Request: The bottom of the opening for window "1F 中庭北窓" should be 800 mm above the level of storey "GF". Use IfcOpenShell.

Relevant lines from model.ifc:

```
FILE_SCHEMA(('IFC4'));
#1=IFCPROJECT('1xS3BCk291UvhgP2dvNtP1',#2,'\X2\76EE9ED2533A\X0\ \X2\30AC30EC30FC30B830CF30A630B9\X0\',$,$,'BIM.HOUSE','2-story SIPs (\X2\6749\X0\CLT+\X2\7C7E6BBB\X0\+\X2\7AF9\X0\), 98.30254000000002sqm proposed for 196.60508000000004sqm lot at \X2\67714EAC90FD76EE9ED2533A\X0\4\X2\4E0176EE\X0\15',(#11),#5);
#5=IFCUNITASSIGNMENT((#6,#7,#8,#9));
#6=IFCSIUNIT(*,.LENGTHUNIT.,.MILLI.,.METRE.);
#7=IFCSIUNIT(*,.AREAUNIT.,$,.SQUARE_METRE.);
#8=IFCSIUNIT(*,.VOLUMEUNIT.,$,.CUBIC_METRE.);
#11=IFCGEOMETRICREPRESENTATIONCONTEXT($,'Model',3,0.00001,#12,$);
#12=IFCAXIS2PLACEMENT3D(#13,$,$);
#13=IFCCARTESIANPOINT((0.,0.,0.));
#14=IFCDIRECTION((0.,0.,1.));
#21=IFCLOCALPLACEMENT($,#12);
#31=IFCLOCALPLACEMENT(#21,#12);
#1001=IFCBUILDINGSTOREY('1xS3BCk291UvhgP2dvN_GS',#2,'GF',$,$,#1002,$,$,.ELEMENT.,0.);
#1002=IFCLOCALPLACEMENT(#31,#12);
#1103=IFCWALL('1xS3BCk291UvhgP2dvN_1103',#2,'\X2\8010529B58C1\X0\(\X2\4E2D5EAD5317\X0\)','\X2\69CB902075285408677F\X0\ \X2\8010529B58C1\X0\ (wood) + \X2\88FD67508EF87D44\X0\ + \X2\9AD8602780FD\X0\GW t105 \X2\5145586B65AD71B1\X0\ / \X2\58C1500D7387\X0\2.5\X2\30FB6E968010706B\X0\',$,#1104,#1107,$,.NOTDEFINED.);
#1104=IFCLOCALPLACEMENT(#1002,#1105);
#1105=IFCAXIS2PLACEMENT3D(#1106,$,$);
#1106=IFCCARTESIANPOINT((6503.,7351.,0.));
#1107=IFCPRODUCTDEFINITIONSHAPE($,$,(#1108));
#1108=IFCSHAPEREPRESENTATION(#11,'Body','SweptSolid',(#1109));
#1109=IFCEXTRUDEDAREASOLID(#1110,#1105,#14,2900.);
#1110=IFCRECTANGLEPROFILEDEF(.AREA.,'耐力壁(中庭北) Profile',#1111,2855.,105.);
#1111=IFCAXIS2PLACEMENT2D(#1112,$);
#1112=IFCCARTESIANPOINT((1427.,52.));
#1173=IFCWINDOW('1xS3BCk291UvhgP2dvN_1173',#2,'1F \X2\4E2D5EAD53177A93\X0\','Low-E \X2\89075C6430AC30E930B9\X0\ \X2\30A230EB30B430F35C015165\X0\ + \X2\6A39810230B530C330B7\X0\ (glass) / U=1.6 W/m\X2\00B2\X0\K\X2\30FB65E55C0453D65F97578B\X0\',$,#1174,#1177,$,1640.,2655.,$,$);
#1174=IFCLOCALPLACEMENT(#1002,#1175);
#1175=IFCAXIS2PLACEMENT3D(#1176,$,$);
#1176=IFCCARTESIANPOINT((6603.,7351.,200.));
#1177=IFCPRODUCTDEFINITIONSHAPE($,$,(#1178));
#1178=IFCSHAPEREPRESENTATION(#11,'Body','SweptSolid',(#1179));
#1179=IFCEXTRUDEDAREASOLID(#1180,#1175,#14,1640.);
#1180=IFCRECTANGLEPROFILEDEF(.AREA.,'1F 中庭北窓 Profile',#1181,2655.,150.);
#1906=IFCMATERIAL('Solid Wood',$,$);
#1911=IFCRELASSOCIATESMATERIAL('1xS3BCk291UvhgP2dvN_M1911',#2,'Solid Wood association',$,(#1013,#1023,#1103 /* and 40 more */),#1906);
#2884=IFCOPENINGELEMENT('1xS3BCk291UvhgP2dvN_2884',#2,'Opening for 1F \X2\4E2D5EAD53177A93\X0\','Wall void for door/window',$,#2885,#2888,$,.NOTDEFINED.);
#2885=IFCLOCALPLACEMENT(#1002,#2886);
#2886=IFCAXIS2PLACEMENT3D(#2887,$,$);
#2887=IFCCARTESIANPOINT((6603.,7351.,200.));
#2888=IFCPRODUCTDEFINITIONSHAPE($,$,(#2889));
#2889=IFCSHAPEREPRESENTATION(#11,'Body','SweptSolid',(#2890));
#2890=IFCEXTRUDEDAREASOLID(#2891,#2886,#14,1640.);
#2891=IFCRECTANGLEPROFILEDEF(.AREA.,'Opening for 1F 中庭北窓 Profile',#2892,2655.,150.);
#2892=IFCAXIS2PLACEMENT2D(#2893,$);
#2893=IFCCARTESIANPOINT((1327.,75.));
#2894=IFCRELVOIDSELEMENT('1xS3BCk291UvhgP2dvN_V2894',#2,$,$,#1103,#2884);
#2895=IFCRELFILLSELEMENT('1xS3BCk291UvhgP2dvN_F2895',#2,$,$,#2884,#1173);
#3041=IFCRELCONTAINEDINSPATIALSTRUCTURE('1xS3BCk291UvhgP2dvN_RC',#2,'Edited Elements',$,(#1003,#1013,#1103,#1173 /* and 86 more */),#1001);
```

```python
import numpy as np
import ifcopenshell
import ifcopenshell.api.geometry
import ifcopenshell.geom
import ifcopenshell.util.element
import ifcopenshell.util.placement
import ifcopenshell.util.shape
import ifcopenshell.util.unit

model = ifcopenshell.open("model.ifc")
unit_scale = ifcopenshell.util.unit.calculate_unit_scale(model)

window = model.by_guid("1xS3BCk291UvhgP2dvN_1173")
opening = window.FillsVoids[0].RelatingOpeningElement
storey = ifcopenshell.util.element.get_container(window, ifc_class="IfcBuildingStorey")
level = ifcopenshell.util.placement.get_local_placement(storey.ObjectPlacement)[2, 3]

# The opening's origin need not be at the sill, so measure its lowest point.
shape = ifcopenshell.geom.create_shape(ifcopenshell.geom.settings(), opening)
bottom = ifcopenshell.util.shape.get_shape_bottom_elevation(shape, shape.geometry) / unit_scale
dz = level + 0.8 / unit_scale - bottom

shift = np.array([0.0, 0.0, dz])
# The window is not placed relative to its opening, so move both.
for product in (opening, window):
    matrix = ifcopenshell.util.placement.get_local_placement(product.ObjectPlacement)
    matrix[:3, 3] += shift
    ifcopenshell.api.geometry.edit_object_placement(model, product=product, matrix=matrix, is_si=False)

print(f"moved by {dz * unit_scale:+.3f} m")

model.write("model_updated.ifc")
```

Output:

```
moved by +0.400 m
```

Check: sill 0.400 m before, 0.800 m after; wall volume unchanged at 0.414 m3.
